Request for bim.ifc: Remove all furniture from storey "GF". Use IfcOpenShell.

First a look at what the model holds.

```python
import ifcopenshell
import ifcopenshell.util.element

model = ifcopenshell.open("bim.ifc")
print(model.schema)
storey = next(s for s in model.by_type("IfcBuildingStorey") if s.Name == "GF")
furniture = [e for e in ifcopenshell.util.element.get_decomposition(storey) if e.is_a("IfcFurnishingElement")]
seen = {}
for e in furniture:
    element_type = ifcopenshell.util.element.get_type(e)
    name = element_type.Name if element_type not in (None, e) else None
    seen[name] = seen.get(name, 0) + 1
for name, count in sorted(seen.items(), key=str):
    print(count, "x", name)
```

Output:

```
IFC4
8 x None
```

```python
import ifcopenshell
import ifcopenshell.api.root
import ifcopenshell.util.element

model = ifcopenshell.open("bim.ifc")

storey = next(s for s in model.by_type("IfcBuildingStorey") if s.Name == "GF")
furniture = [e for e in ifcopenshell.util.element.get_decomposition(storey) if e.is_a("IfcFurnishingElement")]

for e in furniture:
    ifcopenshell.api.root.remove_product(model, product=e)
print(len(furniture), "removed")

model.write("bim_edited.ifc")
```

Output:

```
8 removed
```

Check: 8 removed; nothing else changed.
